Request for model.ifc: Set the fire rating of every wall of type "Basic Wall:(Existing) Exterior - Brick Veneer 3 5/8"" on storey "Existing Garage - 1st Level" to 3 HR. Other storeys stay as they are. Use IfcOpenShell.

First a look at what the model holds.

```python
import ifcopenshell
import ifcopenshell.util.element

model = ifcopenshell.open("model.ifc")
print(model.schema)
storey = next(s for s in model.by_type("IfcBuildingStorey") if s.Name == "Existing Garage - 1st Level")
walls = [e for e in ifcopenshell.util.element.get_decomposition(storey) if e.is_a("IfcWall")]
seen = {}
for e in walls:
    element_type = ifcopenshell.util.element.get_type(e)
    key = (element_type.Name if element_type != e and element_type else None, ifcopenshell.util.element.get_pset(e, "Pset_WallCommon", "FireRating"))
    seen[key] = seen.get(key, 0) + 1
for (name, value), count in sorted(seen.items(), key=str):
    print(count, "x", name, "|", value)
```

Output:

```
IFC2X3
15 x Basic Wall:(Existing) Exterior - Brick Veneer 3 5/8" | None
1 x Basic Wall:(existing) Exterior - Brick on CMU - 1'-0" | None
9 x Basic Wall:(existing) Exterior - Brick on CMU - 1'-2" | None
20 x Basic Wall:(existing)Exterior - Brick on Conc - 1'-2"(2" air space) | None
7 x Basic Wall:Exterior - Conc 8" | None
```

```python
import ifcopenshell
import ifcopenshell.api.pset
import ifcopenshell.util.element

model = ifcopenshell.open("model.ifc")

storey = next(s for s in model.by_type("IfcBuildingStorey") if s.Name == "Existing Garage - 1st Level")
walls = [e for e in ifcopenshell.util.element.get_decomposition(storey) if e.is_a("IfcWall")]

count = 0
for e in walls:
    element_type = ifcopenshell.util.element.get_type(e)
    if element_type in (None, e) or element_type.Name != 'Basic Wall:(Existing) Exterior - Brick Veneer 3 5/8"':
        continue
    # add_pset returns the element's existing set when there is one.
    pset = ifcopenshell.api.pset.add_pset(model, product=e, name="Pset_WallCommon")
    ifcopenshell.api.pset.edit_pset(model, pset=pset, properties={"FireRating": "3 HR"})
    count += 1

print(count, "walls updated")

model.write("model_edited.ifc")
```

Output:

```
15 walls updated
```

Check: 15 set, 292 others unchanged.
